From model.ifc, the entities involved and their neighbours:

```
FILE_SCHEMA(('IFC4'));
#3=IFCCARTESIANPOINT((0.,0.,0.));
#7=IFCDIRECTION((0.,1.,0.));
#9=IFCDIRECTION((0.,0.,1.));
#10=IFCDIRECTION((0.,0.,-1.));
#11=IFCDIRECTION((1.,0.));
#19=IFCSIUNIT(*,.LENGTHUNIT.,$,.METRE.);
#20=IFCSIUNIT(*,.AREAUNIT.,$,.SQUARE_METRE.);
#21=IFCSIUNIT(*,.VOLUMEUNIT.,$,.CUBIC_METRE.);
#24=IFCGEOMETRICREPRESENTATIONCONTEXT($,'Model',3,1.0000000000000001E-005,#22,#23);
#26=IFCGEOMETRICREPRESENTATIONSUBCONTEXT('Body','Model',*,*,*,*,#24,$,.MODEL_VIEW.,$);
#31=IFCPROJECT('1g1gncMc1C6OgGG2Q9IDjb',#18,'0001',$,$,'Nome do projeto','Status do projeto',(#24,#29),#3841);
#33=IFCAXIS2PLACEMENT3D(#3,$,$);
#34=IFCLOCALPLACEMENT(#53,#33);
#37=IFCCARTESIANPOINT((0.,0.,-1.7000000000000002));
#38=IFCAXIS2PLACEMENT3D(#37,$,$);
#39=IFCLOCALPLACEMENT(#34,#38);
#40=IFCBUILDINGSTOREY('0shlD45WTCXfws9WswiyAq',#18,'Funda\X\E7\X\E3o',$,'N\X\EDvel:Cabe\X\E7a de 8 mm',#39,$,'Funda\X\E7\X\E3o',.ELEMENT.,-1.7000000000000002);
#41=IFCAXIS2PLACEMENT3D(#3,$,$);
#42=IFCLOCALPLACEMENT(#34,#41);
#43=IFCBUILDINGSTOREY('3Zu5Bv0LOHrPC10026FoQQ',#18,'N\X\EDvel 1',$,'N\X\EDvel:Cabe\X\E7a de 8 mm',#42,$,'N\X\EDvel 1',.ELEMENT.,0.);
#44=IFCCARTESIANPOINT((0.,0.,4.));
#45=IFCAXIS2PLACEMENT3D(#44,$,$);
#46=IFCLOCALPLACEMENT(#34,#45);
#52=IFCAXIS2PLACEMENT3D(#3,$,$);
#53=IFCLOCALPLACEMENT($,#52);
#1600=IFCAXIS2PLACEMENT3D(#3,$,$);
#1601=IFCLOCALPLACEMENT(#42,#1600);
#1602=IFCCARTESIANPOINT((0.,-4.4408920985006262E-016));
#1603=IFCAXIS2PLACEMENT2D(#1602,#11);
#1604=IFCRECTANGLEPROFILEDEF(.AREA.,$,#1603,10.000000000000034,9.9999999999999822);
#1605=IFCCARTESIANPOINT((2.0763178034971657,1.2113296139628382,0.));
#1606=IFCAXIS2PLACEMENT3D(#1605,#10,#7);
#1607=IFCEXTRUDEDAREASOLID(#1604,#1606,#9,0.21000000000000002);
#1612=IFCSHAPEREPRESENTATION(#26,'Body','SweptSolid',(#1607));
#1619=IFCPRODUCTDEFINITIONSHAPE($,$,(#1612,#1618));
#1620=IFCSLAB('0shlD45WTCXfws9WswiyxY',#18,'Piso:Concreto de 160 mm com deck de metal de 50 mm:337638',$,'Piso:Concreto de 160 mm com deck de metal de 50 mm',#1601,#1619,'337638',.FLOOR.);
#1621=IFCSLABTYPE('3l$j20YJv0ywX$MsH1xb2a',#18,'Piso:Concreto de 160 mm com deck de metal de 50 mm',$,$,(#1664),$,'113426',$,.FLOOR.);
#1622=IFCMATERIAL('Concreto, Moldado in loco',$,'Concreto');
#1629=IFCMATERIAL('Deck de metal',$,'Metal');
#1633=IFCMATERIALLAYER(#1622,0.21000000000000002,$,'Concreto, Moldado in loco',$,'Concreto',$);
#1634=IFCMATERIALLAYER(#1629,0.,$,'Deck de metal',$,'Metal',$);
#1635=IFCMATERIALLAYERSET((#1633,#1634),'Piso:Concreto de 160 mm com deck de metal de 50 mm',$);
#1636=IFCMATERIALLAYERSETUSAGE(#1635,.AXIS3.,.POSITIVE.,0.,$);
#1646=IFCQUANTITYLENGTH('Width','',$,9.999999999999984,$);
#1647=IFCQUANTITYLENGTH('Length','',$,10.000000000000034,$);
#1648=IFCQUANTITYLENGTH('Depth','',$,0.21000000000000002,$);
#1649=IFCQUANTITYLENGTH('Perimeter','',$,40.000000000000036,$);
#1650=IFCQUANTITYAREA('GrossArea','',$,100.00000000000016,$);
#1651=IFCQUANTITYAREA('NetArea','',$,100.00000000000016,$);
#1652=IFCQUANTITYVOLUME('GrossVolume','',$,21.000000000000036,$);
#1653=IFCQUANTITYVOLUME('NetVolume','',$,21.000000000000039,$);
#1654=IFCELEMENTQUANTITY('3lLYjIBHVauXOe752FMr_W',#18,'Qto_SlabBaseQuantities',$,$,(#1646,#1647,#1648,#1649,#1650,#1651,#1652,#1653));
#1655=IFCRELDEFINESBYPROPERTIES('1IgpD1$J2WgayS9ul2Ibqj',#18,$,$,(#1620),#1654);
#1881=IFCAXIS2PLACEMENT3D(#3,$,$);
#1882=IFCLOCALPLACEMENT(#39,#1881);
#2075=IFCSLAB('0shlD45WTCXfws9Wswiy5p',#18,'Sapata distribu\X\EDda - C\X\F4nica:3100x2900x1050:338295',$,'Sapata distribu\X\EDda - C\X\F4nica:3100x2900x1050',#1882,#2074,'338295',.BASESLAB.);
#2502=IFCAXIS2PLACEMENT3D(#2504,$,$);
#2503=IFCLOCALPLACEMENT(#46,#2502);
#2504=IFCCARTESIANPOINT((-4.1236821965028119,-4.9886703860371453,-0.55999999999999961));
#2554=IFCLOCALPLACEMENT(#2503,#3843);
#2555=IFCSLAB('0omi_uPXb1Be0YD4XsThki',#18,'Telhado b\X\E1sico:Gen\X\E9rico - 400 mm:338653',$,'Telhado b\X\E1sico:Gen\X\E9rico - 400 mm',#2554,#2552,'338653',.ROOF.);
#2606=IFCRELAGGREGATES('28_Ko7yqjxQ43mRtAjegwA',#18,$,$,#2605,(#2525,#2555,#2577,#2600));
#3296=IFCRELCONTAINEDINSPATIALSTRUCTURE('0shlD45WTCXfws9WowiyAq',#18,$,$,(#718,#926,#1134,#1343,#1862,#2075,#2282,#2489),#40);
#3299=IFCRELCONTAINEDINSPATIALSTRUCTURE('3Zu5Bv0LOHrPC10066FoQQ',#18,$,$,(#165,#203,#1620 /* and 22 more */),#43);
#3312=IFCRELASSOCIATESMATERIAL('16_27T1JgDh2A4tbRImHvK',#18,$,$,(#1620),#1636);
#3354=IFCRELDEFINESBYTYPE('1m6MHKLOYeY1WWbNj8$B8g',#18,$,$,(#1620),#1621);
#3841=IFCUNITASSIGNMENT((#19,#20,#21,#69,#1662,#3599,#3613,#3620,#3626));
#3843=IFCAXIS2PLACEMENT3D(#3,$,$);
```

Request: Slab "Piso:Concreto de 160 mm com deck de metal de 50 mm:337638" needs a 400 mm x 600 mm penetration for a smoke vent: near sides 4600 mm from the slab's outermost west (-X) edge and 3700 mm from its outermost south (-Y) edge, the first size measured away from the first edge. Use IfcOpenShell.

```python
import numpy as np
import ifcopenshell
import ifcopenshell.api.feature
import ifcopenshell.api.geometry
import ifcopenshell.api.pset
import ifcopenshell.api.root
import ifcopenshell.geom
import ifcopenshell.util.element
import ifcopenshell.util.placement
import ifcopenshell.util.representation
import ifcopenshell.util.shape
import ifcopenshell.util.unit

model = ifcopenshell.open("model.ifc")
unit_scale = ifcopenshell.util.unit.calculate_unit_scale(model)
area_scale = ifcopenshell.util.unit.calculate_unit_scale(model, "AREAUNIT")
volume_scale = ifcopenshell.util.unit.calculate_unit_scale(model, "VOLUMEUNIT")
settings = ifcopenshell.geom.settings()


def volume(element):
    """Net volume in cubic metres, openings subtracted."""
    shape = ifcopenshell.geom.create_shape(settings, element)
    return ifcopenshell.util.shape.get_volume(shape.geometry)


slab = model.by_guid("0shlD45WTCXfws9WswiyxY")
before = volume(slab)

# Extent in the slab's own axes, in metres. The edges named are its -X and -Y sides.
slab_shape = ifcopenshell.geom.create_shape(settings, slab)
vertices = ifcopenshell.util.shape.get_vertices(slab_shape.geometry)
x_min, y_min, bottom = vertices.min(axis=0)
top = vertices[:, 2].max()

opening = ifcopenshell.api.root.create_entity(model, ifc_class="IfcOpeningElement", name="Smoke vent opening", predefined_type="OPENING")
context = ifcopenshell.util.representation.get_context(model, "Model", "Body", "MODEL_VIEW")
width, depth = 0.4, 0.6
outline = [(0.0, 0.0), (width, 0.0), (width, depth), (0.0, depth), (0.0, 0.0)]
# Overshoot both faces by 50 mm so the cut is clean.
shape = ifcopenshell.api.geometry.add_slab_representation(
    model, context=context, depth=top - bottom + 0.1, polyline=outline
)
ifcopenshell.api.geometry.assign_representation(model, product=opening, representation=shape)

matrix = ifcopenshell.util.placement.get_local_placement(slab.ObjectPlacement)
matrix[:, 3] = matrix @ np.append(np.array([x_min + 4.6, y_min + 3.7, bottom - 0.05]) / unit_scale, 1.0)
ifcopenshell.api.geometry.edit_object_placement(model, product=opening, matrix=matrix, is_si=False)
ifcopenshell.api.feature.add_feature(model, feature=opening, element=slab)

after = volume(slab)

# Update the slab's stored quantities.
qto = model.by_id(ifcopenshell.util.element.get_pset(slab, "Qto_SlabBaseQuantities", should_inherit=False)["id"])
ifcopenshell.api.pset.edit_qto(model, qto=qto, properties={
    "NetArea": after / (top - bottom) / area_scale,
    "NetVolume": after / volume_scale,
})

print(f"slab volume {before:.3f} -> {after:.3f} m3")

model.write("model_rev.ifc")
```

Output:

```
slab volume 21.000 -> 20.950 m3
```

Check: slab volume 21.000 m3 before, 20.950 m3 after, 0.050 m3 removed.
